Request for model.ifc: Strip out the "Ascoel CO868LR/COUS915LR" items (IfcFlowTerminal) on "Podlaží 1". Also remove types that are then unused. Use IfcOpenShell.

First a look at what the model holds.

```python
import ifcopenshell
import ifcopenshell.util.element

model = ifcopenshell.open("model.ifc")
print(model.schema)
storey = next(s for s in model.by_type("IfcBuildingStorey") if s.Name == "Podlaží 1")
terminals = [e for e in ifcopenshell.util.element.get_decomposition(storey) if e.is_a("IfcFlowTerminal")]
seen = {}
for e in terminals:
    element_type = ifcopenshell.util.element.get_type(e)
    name = element_type.Name if element_type not in (None, e) else None
    seen[name] = seen.get(name, 0) + 1
for name, count in sorted(seen.items(), key=str):
    print(count, "x", name)
```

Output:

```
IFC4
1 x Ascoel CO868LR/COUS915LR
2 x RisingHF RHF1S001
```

```python
import ifcopenshell
import ifcopenshell.api.root
import ifcopenshell.util.element

model = ifcopenshell.open("model.ifc")

storey = next(s for s in model.by_type("IfcBuildingStorey") if s.Name == "Podlaží 1")
terminals = [e for e in ifcopenshell.util.element.get_decomposition(storey) if e.is_a("IfcFlowTerminal")]
targets = [e for e in terminals if (t := ifcopenshell.util.element.get_type(e)) not in (None, e) and t.Name == "Ascoel CO868LR/COUS915LR"]
types = {ifcopenshell.util.element.get_type(e) for e in targets} - {None, *targets}

for e in targets:
    ifcopenshell.api.root.remove_product(model, product=e)
print(len(targets), "removed")

unused = [t for t in types if not ifcopenshell.util.element.get_types(t)]
for t in unused:
    ifcopenshell.api.root.remove_product(model, product=t)
print(len(unused), "unused types removed")

model.write("model_edited.ifc")
```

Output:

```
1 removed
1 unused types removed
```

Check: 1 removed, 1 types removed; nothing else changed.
